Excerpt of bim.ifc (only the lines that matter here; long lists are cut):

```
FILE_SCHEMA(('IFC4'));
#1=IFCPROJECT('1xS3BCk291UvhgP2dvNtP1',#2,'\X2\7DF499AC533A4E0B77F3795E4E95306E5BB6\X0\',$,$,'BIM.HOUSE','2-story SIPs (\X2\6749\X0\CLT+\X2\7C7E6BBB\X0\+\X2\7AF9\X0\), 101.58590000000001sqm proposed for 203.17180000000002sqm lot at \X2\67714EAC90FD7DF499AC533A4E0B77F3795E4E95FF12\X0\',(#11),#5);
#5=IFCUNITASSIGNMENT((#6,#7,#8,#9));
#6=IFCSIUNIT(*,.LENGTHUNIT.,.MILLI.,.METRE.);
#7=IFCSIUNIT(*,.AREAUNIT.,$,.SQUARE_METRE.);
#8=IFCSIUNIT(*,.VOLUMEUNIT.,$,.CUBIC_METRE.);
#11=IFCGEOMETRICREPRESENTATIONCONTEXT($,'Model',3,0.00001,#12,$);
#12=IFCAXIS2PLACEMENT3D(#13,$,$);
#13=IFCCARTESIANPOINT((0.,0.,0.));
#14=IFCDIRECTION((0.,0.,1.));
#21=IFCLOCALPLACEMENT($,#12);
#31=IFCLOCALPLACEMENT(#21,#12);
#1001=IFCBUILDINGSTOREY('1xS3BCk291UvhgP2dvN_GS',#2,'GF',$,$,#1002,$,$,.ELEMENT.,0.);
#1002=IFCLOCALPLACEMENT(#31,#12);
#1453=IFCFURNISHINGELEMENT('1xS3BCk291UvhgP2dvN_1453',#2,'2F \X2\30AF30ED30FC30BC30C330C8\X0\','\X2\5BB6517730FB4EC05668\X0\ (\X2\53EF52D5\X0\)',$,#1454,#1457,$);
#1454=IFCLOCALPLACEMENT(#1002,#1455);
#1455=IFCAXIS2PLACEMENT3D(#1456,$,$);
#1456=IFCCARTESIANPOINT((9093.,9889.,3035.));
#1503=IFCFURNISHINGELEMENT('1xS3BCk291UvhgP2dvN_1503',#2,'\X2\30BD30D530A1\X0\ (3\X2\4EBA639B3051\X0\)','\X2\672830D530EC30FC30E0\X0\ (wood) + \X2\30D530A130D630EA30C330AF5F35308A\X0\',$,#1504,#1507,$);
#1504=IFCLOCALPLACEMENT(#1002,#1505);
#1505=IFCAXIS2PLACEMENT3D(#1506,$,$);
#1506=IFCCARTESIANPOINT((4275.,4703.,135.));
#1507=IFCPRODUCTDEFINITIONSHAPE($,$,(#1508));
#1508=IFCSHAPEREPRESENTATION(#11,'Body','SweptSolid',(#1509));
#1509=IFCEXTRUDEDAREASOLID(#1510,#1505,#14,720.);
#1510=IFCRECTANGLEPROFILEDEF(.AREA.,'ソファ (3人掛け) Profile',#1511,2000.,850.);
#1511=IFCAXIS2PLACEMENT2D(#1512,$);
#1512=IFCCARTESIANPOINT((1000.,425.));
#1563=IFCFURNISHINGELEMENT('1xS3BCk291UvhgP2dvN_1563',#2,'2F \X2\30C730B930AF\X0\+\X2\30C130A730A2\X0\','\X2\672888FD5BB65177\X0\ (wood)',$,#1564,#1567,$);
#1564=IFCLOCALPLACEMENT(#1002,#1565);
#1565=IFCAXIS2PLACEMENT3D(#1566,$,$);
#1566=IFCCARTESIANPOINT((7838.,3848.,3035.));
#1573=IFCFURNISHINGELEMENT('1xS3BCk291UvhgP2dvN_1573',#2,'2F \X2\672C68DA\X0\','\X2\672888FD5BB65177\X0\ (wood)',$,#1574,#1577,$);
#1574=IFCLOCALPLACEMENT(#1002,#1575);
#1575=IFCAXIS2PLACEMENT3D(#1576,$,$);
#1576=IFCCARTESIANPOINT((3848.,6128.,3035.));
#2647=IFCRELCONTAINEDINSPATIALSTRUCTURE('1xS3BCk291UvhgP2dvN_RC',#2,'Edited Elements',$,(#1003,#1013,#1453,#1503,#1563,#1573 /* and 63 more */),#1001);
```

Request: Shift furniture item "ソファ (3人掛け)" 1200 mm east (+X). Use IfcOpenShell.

```python
import ifcopenshell
import ifcopenshell.api.geometry
import ifcopenshell.util.placement
import ifcopenshell.util.unit

model = ifcopenshell.open("bim.ifc")
unit_scale = ifcopenshell.util.unit.calculate_unit_scale(model)

item = model.by_id(1503)
matrix = ifcopenshell.util.placement.get_local_placement(item.ObjectPlacement)
matrix[0, 3] += 1.2 / unit_scale
ifcopenshell.api.geometry.edit_object_placement(model, product=item, matrix=matrix, is_si=False)

print(ifcopenshell.util.placement.get_local_placement(item.ObjectPlacement).round(3) + 0.0)

model.write("bim_edited.ifc")
```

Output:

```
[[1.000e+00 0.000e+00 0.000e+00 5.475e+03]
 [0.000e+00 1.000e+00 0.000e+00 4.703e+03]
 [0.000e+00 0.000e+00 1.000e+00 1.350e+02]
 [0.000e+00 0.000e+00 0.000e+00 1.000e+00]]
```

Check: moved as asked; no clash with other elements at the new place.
